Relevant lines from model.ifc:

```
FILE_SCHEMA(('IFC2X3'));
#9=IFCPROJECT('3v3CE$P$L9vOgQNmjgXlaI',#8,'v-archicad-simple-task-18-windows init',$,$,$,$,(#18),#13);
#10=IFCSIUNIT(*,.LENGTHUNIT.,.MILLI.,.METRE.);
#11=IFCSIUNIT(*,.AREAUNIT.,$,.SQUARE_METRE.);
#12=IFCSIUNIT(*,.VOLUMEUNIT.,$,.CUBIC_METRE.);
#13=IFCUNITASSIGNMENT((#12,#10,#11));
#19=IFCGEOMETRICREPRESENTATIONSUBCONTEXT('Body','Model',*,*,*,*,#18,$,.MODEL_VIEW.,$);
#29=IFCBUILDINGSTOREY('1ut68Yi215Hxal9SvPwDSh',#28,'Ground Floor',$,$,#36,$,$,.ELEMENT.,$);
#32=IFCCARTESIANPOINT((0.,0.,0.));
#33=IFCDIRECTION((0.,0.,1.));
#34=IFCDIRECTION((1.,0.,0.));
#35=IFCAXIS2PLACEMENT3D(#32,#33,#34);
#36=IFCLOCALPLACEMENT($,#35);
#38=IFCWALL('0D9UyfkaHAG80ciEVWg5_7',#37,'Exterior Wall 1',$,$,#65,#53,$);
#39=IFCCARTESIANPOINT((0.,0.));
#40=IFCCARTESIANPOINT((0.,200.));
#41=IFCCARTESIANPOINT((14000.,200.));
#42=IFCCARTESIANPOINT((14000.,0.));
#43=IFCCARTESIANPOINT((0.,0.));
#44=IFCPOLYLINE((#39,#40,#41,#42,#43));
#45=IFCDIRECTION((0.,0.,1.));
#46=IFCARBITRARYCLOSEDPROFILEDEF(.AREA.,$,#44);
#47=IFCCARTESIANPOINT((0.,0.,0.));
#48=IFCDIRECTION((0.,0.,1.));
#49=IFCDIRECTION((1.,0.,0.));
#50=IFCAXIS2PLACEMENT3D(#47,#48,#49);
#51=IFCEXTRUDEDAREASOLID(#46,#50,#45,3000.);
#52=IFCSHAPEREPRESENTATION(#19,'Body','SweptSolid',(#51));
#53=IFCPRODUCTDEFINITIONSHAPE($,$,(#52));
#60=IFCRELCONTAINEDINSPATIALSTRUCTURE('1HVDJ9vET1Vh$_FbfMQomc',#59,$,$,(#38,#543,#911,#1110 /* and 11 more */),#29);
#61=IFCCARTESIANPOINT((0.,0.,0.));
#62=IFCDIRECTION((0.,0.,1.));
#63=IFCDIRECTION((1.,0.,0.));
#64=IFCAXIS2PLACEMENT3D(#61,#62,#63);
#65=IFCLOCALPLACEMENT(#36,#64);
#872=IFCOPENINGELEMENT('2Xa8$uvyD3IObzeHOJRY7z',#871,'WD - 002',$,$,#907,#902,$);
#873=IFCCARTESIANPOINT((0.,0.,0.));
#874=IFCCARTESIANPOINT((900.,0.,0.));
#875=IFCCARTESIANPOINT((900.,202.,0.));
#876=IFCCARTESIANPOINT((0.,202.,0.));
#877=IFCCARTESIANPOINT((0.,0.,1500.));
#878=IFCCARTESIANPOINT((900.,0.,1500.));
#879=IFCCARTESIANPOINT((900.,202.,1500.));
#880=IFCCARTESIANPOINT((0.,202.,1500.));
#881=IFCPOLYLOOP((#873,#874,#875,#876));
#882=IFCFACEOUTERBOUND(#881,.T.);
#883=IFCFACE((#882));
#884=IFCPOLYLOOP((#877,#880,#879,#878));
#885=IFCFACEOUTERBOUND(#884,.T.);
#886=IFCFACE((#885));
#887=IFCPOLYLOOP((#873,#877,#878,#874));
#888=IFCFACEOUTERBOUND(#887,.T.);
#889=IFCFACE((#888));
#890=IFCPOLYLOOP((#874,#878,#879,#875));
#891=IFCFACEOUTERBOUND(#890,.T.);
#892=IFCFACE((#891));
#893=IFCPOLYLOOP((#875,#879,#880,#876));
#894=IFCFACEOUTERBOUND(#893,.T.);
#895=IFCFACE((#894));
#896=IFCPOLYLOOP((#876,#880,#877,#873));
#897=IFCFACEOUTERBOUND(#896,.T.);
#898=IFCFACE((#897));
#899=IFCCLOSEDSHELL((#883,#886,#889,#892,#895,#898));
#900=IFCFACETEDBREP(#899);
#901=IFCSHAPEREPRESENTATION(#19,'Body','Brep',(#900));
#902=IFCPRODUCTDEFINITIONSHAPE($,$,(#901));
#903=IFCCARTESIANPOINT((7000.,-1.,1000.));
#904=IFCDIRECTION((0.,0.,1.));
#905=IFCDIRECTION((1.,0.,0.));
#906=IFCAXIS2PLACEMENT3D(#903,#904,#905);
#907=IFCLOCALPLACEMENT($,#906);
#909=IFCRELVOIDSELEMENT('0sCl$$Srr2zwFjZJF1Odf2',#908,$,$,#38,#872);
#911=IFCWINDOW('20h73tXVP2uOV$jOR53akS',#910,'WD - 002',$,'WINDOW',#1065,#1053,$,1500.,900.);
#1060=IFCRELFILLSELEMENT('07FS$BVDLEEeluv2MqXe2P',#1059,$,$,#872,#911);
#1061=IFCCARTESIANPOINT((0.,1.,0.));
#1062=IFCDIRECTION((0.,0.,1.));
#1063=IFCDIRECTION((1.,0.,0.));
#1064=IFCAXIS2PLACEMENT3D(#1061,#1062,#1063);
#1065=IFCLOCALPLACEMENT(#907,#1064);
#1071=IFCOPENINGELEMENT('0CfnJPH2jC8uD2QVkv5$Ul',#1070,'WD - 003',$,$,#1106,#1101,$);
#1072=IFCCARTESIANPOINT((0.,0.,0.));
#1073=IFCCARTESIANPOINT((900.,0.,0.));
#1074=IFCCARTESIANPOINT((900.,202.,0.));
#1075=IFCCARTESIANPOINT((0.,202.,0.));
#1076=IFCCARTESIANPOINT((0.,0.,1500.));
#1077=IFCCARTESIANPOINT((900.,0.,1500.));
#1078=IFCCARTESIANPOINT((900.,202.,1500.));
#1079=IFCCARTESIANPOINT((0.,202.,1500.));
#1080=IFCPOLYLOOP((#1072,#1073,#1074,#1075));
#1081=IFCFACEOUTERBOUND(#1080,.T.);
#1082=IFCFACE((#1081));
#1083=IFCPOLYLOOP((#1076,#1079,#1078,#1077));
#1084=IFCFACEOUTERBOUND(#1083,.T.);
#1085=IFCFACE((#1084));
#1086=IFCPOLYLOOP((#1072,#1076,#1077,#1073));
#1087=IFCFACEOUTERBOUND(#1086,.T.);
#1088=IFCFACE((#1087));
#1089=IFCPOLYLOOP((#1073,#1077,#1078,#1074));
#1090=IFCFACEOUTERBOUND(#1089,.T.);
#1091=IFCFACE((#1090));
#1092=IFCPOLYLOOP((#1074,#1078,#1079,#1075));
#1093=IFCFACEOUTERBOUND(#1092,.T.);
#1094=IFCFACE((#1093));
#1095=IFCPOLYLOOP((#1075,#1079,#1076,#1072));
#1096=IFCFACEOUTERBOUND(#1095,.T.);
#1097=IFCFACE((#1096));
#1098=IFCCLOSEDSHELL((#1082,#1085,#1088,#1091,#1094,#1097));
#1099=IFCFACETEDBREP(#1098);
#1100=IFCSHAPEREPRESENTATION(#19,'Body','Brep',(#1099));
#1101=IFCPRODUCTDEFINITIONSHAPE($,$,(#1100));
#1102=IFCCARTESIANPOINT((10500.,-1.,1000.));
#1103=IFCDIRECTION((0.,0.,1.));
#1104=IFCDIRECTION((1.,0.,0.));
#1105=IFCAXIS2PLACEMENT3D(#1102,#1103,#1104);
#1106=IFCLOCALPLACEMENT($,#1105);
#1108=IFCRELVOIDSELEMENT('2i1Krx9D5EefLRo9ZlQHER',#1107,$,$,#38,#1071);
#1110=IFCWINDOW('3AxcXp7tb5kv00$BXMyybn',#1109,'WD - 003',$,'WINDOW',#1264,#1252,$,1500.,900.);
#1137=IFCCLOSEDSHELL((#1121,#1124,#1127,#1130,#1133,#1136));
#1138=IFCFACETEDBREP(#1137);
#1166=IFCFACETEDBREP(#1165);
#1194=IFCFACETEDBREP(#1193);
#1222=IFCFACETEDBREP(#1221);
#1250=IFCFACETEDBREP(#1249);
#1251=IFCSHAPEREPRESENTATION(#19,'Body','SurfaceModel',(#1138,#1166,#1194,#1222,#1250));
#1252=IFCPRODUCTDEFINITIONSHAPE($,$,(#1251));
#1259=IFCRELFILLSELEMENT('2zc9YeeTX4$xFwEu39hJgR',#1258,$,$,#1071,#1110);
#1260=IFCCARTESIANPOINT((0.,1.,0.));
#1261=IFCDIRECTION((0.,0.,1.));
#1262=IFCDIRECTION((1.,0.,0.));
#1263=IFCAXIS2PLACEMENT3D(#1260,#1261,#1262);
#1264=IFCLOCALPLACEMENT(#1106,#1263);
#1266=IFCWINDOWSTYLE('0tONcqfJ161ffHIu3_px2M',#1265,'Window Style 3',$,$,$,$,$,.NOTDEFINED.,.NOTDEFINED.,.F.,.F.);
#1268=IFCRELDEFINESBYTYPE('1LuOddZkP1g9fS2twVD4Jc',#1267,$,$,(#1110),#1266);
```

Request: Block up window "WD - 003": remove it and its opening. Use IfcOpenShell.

```python
import ifcopenshell
import ifcopenshell.api.feature
import ifcopenshell.api.root
import ifcopenshell.geom
import ifcopenshell.util.shape

model = ifcopenshell.open("model.ifc")
settings = ifcopenshell.geom.settings()


def volume(element):
    """Net volume in cubic metres, openings subtracted."""
    shape = ifcopenshell.geom.create_shape(settings, element)
    return ifcopenshell.util.shape.get_volume(shape.geometry)


window = model.by_guid("3AxcXp7tb5kv00$BXMyybn")
opening = window.FillsVoids[0].RelatingOpeningElement
wall = opening.VoidsElements[0].RelatingBuildingElement
before = volume(wall)

ifcopenshell.api.root.remove_product(model, product=window)
ifcopenshell.api.feature.remove_feature(model, feature=opening)

after = volume(wall)

print(f"wall volume {before:.3f} -> {after:.3f} m3")

model.write("model_updated.ifc")
```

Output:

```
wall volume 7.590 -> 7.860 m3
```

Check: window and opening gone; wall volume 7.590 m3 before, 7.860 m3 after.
